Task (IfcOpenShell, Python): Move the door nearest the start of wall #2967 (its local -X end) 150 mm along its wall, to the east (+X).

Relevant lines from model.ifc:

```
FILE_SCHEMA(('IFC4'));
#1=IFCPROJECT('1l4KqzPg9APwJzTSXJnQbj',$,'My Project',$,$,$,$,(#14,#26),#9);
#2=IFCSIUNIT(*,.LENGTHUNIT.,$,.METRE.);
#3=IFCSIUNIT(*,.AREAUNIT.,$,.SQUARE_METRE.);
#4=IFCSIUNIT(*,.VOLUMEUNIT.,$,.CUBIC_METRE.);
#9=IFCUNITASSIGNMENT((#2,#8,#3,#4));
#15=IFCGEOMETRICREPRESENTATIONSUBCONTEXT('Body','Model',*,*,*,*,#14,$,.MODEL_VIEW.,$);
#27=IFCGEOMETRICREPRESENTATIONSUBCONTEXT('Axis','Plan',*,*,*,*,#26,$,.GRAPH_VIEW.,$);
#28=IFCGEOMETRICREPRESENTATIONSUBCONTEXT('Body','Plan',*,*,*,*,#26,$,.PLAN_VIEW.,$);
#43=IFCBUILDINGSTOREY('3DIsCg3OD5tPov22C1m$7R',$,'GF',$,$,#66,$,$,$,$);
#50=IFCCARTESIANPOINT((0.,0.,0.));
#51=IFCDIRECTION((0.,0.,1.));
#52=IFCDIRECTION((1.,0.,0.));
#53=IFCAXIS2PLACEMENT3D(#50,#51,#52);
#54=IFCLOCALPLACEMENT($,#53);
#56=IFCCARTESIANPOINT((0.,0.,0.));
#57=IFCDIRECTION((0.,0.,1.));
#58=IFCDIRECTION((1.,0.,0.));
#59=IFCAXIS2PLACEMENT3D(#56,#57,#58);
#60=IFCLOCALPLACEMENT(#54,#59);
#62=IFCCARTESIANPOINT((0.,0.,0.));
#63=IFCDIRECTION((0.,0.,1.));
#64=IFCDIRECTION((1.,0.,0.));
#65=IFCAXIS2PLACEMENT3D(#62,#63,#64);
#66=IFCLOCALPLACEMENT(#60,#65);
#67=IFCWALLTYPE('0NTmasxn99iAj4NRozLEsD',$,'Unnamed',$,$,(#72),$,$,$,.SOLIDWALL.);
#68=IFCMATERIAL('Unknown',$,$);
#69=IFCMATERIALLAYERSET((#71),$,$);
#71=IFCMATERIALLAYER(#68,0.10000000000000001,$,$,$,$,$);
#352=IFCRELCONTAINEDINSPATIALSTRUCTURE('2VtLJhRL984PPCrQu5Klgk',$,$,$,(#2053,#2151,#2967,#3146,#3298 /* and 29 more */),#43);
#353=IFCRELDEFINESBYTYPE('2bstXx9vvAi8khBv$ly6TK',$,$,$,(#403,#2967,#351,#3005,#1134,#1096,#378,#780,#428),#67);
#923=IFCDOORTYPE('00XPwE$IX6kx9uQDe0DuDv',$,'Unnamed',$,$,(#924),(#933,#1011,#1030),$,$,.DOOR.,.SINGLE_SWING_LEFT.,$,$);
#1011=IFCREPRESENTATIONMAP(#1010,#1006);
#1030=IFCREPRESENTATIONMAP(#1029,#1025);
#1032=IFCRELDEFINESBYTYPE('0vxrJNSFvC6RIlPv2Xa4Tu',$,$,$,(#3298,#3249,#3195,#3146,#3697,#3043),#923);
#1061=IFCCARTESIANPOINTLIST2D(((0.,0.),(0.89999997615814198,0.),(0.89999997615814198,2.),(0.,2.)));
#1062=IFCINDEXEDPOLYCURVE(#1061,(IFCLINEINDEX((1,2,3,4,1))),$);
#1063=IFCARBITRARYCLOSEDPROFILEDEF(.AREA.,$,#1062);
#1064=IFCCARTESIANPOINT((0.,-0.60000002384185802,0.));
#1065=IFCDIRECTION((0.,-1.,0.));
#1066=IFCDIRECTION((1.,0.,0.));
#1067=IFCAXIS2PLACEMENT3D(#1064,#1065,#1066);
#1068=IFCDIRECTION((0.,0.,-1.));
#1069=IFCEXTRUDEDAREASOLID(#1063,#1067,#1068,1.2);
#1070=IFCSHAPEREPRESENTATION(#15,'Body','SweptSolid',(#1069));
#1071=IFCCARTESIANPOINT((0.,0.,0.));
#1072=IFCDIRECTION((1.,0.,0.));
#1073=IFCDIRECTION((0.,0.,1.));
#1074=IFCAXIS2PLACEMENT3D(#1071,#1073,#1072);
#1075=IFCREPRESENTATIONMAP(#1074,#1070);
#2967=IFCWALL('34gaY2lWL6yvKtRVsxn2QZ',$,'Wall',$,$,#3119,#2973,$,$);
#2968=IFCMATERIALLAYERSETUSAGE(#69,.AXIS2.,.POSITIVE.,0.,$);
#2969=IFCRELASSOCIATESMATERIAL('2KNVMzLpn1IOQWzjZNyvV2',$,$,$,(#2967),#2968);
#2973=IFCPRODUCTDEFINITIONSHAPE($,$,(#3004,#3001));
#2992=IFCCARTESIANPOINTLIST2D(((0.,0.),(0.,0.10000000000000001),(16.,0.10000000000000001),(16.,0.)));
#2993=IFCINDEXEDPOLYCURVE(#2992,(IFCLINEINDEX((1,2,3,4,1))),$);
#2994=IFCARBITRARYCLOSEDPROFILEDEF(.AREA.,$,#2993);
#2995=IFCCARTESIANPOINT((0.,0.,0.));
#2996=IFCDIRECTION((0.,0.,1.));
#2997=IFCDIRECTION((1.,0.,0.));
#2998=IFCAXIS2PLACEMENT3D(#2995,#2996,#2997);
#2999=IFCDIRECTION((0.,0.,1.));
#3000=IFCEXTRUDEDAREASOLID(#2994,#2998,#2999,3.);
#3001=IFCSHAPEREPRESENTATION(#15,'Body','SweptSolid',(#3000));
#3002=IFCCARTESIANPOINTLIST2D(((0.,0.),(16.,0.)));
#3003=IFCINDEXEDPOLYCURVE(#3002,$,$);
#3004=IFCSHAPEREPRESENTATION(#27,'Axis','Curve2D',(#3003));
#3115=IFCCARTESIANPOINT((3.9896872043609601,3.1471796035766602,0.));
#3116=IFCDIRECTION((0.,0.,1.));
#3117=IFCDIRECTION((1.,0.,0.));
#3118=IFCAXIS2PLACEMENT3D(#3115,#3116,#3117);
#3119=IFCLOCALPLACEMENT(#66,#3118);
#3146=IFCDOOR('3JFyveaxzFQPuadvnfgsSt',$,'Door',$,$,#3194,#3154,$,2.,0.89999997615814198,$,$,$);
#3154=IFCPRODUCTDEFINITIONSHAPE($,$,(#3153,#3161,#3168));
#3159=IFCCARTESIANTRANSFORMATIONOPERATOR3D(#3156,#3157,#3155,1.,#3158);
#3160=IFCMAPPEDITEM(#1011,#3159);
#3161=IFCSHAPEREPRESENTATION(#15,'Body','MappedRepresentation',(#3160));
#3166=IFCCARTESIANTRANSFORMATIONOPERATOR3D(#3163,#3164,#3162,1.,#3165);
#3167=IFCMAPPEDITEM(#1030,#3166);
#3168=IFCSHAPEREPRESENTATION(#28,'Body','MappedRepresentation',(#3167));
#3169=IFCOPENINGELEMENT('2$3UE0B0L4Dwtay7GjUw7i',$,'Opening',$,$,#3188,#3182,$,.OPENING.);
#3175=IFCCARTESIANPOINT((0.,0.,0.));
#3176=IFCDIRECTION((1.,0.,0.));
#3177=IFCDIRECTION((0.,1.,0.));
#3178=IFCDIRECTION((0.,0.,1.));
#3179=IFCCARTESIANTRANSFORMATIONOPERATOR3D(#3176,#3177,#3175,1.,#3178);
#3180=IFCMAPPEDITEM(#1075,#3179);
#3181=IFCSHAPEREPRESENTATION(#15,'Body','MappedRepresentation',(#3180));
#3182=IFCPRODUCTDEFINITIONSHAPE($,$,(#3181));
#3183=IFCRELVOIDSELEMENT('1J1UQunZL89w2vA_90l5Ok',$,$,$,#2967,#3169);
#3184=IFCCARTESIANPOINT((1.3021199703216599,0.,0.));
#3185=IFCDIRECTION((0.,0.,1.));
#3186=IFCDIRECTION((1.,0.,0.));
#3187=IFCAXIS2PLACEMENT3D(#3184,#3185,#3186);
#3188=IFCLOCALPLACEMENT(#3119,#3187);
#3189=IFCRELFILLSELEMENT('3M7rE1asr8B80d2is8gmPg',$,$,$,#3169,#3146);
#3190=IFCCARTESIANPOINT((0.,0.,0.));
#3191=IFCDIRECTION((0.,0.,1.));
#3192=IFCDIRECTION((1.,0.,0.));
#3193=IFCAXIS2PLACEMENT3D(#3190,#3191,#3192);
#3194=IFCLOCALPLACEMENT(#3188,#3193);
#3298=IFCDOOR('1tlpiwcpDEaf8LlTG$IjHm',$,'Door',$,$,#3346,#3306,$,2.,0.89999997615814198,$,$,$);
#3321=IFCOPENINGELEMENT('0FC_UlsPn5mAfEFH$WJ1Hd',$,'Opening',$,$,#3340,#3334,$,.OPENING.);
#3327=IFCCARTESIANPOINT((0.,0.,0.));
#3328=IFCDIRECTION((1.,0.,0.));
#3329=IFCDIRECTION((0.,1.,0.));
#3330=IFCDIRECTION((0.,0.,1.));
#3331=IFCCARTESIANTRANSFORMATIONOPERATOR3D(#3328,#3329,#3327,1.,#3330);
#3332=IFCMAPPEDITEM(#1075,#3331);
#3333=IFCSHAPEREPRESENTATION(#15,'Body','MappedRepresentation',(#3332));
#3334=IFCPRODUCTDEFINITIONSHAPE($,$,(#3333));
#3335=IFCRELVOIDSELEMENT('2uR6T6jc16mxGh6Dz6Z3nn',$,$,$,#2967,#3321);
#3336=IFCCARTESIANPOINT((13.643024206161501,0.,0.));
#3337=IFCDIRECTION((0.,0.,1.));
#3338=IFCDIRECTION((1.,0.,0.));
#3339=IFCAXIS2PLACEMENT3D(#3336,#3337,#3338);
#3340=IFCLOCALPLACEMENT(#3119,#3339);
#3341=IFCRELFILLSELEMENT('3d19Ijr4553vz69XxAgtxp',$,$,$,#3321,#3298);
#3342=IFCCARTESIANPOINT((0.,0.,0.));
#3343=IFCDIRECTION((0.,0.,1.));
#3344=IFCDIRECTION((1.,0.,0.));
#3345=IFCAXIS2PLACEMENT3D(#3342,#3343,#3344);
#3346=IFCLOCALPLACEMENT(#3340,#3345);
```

```python
import ifcopenshell
import ifcopenshell.api.geometry
import ifcopenshell.util.placement

model = ifcopenshell.open("model.ifc")

door = model.by_guid("3JFyveaxzFQPuadvnfgsSt")
opening = door.FillsVoids[0].RelatingOpeningElement
wall = opening.VoidsElements[0].RelatingBuildingElement

wall_matrix = ifcopenshell.util.placement.get_local_placement(wall.ObjectPlacement)
shift = wall_matrix[:3, 0] * 0.15
before = ifcopenshell.util.placement.get_local_placement(door.ObjectPlacement)[:3, 3].copy()

# The door is placed relative to its opening, so it follows when the opening moves.
matrix = ifcopenshell.util.placement.get_local_placement(opening.ObjectPlacement)
matrix[:3, 3] += shift
ifcopenshell.api.geometry.edit_object_placement(
    model, product=opening, matrix=matrix, is_si=False, should_transform_children=True
)

after = ifcopenshell.util.placement.get_local_placement(door.ObjectPlacement)[:3, 3]
print("door moved by", (after - before).round(3) + 0.0)

model.write("model_edited.ifc")
```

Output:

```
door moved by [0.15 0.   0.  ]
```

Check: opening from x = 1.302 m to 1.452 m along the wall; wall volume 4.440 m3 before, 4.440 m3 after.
